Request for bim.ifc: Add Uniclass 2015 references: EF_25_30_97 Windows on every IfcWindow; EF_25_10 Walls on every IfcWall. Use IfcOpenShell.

First a look at what the model holds.

```python
import ifcopenshell

model = ifcopenshell.open("bim.ifc")
print(model.schema)
print("classifications:", [c.Name for c in model.by_type("IfcClassification")])
for ifc_class in ("IfcDoor", "IfcRoof", "IfcStair", "IfcWall", "IfcWindow"):
    print(ifc_class, len(model.by_type(ifc_class)))
```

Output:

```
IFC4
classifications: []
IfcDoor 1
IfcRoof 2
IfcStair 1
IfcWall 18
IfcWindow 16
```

```python
import ifcopenshell
import ifcopenshell.api.classification

model = ifcopenshell.open("bim.ifc")

system = ifcopenshell.api.classification.add_classification(model, classification="Uniclass 2015")

codes = {
    "IfcWindow": ("EF_25_30_97", "Windows"),
    "IfcWall": ("EF_25_10", "Walls"),
}
for ifc_class, (code, name) in codes.items():
    products = model.by_type(ifc_class)
    ifcopenshell.api.classification.add_reference(
        model, products=products, classification=system, identification=code, name=name
    )
    print(code, len(products))

model.write("bim_v2.ifc")
```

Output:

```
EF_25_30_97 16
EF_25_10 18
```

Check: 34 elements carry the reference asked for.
